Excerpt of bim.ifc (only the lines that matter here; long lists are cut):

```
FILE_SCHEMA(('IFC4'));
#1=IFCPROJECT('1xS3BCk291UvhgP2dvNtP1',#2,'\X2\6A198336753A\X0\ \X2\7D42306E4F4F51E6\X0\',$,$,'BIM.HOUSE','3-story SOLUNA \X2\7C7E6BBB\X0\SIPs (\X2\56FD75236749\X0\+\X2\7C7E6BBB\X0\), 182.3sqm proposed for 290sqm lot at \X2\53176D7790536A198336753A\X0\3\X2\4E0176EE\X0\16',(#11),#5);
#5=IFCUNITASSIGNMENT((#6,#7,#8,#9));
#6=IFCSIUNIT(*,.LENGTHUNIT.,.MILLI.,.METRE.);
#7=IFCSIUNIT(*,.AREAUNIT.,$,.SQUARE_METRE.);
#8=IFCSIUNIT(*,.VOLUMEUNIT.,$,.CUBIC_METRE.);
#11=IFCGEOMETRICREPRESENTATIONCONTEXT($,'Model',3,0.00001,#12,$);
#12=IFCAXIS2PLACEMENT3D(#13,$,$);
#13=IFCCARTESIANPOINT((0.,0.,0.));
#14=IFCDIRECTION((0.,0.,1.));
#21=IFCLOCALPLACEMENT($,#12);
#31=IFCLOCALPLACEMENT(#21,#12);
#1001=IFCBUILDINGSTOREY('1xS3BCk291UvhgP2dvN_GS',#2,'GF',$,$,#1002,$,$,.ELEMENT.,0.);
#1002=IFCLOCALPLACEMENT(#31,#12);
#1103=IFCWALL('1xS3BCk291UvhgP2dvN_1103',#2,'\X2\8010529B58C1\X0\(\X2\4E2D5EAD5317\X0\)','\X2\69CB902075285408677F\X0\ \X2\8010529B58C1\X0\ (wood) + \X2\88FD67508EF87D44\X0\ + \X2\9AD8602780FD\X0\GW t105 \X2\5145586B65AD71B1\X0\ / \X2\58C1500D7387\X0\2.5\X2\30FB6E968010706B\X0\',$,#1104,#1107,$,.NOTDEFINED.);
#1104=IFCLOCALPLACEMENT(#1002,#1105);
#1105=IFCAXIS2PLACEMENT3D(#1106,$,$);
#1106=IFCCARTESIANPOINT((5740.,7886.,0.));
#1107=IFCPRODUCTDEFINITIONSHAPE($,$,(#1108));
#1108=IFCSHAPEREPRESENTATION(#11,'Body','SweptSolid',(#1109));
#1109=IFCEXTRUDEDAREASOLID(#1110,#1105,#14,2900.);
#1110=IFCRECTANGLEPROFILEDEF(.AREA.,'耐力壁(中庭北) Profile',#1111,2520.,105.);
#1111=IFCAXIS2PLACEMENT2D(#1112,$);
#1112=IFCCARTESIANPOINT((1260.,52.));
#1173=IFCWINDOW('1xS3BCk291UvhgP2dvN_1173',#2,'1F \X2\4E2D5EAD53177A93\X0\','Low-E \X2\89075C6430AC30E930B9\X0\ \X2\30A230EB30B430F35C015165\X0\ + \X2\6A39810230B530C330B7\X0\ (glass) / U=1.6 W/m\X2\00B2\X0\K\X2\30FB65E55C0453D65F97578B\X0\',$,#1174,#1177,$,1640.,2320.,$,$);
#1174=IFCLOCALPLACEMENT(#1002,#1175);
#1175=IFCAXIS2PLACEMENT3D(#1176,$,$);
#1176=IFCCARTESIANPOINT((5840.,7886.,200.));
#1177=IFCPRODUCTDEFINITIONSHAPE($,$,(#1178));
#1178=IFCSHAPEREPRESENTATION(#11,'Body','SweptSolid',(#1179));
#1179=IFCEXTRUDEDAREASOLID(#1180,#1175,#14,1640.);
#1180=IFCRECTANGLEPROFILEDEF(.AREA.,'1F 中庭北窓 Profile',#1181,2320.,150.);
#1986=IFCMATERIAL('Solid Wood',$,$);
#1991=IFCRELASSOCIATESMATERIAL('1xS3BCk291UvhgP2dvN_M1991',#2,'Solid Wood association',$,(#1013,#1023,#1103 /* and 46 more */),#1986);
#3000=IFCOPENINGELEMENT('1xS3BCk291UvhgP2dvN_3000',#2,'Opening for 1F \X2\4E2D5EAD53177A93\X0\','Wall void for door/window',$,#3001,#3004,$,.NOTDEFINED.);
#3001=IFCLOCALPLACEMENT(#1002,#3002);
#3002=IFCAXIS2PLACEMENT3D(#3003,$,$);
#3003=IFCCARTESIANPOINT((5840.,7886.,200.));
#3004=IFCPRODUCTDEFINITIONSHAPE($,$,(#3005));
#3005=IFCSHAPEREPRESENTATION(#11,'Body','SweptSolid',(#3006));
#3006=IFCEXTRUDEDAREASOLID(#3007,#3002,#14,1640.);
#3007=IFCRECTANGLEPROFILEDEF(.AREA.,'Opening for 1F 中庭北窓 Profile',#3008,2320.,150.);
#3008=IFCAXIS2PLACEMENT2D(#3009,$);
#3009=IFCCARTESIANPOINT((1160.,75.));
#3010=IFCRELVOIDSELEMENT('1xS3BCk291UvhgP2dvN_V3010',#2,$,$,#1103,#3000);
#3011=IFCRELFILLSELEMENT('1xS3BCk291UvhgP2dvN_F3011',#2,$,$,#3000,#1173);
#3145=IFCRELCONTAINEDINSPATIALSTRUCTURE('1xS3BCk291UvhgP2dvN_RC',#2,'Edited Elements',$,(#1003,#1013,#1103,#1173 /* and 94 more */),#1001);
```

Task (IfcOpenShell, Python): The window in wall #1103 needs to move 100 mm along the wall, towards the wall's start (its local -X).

```python
import ifcopenshell
import ifcopenshell.api.geometry
import ifcopenshell.util.placement

model = ifcopenshell.open("bim.ifc")

window = model.by_guid("1xS3BCk291UvhgP2dvN_1173")
opening = window.FillsVoids[0].RelatingOpeningElement
wall = opening.VoidsElements[0].RelatingBuildingElement

wall_matrix = ifcopenshell.util.placement.get_local_placement(wall.ObjectPlacement)
shift = wall_matrix[:3, 0] * -100.0
before = ifcopenshell.util.placement.get_local_placement(window.ObjectPlacement)[:3, 3].copy()

# The window is not placed relative to its opening, so move both.
for product in (opening, window):
    matrix = ifcopenshell.util.placement.get_local_placement(product.ObjectPlacement)
    matrix[:3, 3] += shift
    ifcopenshell.api.geometry.edit_object_placement(model, product=product, matrix=matrix, is_si=False)

after = ifcopenshell.util.placement.get_local_placement(window.ObjectPlacement)[:3, 3]
print("window moved by", (after - before).round(3) + 0.0)

model.write("bim_edited.ifc")
```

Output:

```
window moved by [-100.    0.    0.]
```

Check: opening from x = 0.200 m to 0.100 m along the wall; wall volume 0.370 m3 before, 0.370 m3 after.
